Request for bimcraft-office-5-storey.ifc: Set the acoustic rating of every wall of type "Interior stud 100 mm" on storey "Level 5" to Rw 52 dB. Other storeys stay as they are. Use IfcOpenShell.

First a look at what the model holds.

```python
import ifcopenshell
import ifcopenshell.util.element

model = ifcopenshell.open("bimcraft-office-5-storey.ifc")
print(model.schema)
storey = next(s for s in model.by_type("IfcBuildingStorey") if s.Name == "Level 5")
walls = [e for e in ifcopenshell.util.element.get_decomposition(storey) if e.is_a("IfcWall")]
seen = {}
for e in walls:
    element_type = ifcopenshell.util.element.get_type(e)
    key = (element_type.Name if element_type != e and element_type else None, ifcopenshell.util.element.get_pset(e, "Pset_WallCommon", "AcousticRating"))
    seen[key] = seen.get(key, 0) + 1
for (name, value), count in sorted(seen.items(), key=str):
    print(count, "x", name, "|", value)
```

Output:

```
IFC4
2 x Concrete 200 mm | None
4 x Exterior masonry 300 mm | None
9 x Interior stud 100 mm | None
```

```python
import ifcopenshell
import ifcopenshell.api.pset
import ifcopenshell.util.element

model = ifcopenshell.open("bimcraft-office-5-storey.ifc")

storey = next(s for s in model.by_type("IfcBuildingStorey") if s.Name == "Level 5")
walls = [e for e in ifcopenshell.util.element.get_decomposition(storey) if e.is_a("IfcWall")]

count = 0
for e in walls:
    element_type = ifcopenshell.util.element.get_type(e)
    if element_type in (None, e) or element_type.Name != "Interior stud 100 mm":
        continue
    # add_pset returns the element's existing set when there is one.
    pset = ifcopenshell.api.pset.add_pset(model, product=e, name="Pset_WallCommon")
    ifcopenshell.api.pset.edit_pset(model, pset=pset, properties={"AcousticRating": "Rw 52 dB"})
    count += 1

print(count, "walls updated")

model.write("bimcraft-office-5-storey-out.ifc")
```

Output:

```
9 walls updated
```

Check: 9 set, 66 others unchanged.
